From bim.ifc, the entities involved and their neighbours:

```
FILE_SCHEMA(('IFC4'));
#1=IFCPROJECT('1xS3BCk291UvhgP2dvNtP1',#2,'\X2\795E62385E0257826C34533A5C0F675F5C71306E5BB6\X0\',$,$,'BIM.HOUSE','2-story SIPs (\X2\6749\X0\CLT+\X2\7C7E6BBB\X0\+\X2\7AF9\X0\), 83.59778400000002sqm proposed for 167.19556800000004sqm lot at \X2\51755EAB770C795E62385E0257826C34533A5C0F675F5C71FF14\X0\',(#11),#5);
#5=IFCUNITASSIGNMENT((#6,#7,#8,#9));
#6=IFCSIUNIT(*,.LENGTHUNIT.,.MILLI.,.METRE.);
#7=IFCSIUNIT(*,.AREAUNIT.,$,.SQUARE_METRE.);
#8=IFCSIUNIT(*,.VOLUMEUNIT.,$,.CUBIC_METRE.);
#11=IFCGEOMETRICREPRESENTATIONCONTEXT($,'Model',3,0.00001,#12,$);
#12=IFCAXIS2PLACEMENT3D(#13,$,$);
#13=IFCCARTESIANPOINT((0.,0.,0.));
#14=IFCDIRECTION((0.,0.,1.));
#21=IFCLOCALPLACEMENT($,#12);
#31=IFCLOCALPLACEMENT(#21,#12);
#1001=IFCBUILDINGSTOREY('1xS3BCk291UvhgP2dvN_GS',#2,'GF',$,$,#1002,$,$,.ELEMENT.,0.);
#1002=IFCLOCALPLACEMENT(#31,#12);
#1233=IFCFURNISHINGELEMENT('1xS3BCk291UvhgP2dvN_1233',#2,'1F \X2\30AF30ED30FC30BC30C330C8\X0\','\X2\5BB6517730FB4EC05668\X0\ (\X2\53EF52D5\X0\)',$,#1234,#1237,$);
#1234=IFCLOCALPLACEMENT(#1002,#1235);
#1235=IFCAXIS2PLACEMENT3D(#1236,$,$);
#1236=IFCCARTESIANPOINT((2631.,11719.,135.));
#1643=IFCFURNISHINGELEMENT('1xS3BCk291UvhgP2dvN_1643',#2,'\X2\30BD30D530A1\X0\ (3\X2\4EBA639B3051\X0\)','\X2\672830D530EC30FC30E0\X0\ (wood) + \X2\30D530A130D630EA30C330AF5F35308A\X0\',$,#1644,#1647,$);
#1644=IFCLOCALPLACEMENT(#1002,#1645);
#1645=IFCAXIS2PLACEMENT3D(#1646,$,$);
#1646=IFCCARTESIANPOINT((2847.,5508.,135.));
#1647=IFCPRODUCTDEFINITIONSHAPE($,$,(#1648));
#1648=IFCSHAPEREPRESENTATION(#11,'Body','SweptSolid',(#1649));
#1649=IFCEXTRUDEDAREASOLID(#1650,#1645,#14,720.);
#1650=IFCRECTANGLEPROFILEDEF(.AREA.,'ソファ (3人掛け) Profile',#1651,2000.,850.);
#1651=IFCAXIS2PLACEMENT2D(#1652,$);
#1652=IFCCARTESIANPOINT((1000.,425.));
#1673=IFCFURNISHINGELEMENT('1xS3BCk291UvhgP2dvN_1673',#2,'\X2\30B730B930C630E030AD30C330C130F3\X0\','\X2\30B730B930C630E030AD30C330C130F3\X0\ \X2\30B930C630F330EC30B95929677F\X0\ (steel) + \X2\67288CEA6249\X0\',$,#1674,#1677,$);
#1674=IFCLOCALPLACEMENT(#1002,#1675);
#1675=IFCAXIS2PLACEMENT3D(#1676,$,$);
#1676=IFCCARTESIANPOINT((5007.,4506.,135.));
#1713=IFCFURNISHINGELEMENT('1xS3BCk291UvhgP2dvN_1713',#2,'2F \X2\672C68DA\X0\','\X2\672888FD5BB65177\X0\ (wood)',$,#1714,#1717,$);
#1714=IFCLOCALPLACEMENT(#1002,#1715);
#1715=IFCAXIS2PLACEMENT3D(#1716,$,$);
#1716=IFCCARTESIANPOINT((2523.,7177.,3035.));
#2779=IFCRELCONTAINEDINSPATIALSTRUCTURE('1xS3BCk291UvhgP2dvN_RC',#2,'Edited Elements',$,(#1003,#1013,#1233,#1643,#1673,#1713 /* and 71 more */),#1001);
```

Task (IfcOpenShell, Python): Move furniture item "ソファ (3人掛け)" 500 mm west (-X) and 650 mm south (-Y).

```python
import ifcopenshell
import ifcopenshell.api.geometry
import ifcopenshell.util.placement

model = ifcopenshell.open("bim.ifc")

item = model.by_id(1643)
matrix = ifcopenshell.util.placement.get_local_placement(item.ObjectPlacement)
matrix[0, 3] -= 500.0
matrix[1, 3] -= 650.0
ifcopenshell.api.geometry.edit_object_placement(model, product=item, matrix=matrix, is_si=False)

print(ifcopenshell.util.placement.get_local_placement(item.ObjectPlacement).round(3) + 0.0)

model.write("bim_updated.ifc")
```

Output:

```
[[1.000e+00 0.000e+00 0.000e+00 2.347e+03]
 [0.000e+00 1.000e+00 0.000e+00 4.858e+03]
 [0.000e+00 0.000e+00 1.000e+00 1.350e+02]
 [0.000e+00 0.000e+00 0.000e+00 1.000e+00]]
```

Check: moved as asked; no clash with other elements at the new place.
